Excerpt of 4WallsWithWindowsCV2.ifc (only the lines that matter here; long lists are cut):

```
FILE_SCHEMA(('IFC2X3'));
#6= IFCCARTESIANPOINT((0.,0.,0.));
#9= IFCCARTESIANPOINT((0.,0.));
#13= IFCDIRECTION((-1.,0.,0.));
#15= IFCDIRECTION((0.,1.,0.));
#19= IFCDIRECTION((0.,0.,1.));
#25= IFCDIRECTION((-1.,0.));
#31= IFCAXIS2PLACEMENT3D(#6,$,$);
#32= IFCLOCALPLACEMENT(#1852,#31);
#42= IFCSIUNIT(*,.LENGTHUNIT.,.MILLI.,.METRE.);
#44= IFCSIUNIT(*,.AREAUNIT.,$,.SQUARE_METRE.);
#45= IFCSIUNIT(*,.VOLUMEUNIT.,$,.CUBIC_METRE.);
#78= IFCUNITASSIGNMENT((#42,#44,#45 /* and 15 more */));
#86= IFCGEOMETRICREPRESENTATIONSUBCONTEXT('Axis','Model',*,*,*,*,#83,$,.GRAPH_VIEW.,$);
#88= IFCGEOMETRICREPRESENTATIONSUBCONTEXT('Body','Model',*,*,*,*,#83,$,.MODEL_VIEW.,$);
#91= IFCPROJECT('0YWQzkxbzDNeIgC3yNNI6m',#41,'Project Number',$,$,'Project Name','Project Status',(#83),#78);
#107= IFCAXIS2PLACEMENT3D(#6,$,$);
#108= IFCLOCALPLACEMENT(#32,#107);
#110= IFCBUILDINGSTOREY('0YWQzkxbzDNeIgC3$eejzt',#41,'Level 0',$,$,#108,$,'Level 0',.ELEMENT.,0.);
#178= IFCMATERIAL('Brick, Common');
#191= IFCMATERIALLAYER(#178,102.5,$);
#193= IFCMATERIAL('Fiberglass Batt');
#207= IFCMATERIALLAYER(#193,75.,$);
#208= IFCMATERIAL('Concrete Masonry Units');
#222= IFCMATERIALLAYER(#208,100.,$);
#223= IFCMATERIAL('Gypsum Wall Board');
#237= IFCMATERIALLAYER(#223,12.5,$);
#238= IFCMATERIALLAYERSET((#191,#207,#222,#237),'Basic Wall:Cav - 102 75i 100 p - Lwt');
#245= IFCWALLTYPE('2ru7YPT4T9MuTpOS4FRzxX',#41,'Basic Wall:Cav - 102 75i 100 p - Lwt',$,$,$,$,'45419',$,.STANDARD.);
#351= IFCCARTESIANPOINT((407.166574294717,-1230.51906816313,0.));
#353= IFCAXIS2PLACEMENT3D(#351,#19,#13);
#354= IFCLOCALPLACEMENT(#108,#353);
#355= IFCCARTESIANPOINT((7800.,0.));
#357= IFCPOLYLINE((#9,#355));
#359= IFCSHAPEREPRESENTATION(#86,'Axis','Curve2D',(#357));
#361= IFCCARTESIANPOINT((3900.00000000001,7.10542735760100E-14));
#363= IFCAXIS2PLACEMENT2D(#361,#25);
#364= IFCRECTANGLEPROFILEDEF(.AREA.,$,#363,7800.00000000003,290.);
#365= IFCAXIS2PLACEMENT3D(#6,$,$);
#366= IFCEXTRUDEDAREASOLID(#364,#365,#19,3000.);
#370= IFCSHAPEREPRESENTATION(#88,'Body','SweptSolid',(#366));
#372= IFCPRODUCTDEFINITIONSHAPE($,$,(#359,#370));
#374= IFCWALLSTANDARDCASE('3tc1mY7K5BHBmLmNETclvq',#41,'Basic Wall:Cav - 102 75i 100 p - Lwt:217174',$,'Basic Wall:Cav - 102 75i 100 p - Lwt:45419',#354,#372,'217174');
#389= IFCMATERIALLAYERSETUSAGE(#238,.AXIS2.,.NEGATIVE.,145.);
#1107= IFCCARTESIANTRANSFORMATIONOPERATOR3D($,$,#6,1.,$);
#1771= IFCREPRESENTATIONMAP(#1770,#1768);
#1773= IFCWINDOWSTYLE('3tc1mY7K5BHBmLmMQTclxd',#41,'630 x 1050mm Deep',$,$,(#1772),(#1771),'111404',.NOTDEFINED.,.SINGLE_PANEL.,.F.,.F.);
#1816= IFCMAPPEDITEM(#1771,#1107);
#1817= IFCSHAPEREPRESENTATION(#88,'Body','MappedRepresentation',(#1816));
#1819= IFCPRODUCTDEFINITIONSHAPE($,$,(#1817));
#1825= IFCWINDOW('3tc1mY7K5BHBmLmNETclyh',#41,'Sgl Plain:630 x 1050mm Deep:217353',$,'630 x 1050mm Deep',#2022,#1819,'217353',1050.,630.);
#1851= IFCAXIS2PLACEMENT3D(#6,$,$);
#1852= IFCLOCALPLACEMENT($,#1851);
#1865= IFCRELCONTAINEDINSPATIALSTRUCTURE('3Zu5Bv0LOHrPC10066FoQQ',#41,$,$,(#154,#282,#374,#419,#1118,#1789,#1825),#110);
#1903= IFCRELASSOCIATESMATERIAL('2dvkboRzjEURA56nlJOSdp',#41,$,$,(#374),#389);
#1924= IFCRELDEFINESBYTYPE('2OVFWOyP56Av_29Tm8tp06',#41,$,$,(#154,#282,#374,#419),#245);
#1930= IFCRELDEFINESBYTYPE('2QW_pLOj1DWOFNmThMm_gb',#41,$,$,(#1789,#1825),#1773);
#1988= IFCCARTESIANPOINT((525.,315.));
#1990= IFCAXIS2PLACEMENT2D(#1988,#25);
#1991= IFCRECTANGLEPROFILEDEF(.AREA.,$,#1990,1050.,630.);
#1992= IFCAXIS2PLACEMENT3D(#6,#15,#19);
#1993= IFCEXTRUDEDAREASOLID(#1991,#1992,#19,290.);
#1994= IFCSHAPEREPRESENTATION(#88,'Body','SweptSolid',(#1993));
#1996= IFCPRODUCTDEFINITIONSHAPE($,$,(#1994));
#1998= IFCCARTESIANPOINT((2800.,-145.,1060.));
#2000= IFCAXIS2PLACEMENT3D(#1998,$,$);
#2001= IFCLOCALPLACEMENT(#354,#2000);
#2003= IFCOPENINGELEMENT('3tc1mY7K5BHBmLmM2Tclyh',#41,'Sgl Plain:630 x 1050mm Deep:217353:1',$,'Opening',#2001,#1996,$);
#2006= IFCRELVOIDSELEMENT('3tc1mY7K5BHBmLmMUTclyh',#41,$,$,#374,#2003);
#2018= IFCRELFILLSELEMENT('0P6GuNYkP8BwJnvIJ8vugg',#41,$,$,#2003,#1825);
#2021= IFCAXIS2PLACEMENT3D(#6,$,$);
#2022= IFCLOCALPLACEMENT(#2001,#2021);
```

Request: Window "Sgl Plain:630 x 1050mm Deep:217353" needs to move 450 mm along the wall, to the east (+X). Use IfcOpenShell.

```python
import ifcopenshell
import ifcopenshell.api.geometry
import ifcopenshell.util.placement

model = ifcopenshell.open("4WallsWithWindowsCV2.ifc")

window = model.by_guid("3tc1mY7K5BHBmLmNETclyh")
opening = window.FillsVoids[0].RelatingOpeningElement
wall = opening.VoidsElements[0].RelatingBuildingElement

wall_matrix = ifcopenshell.util.placement.get_local_placement(wall.ObjectPlacement)
shift = wall_matrix[:3, 0] * -450.0
before = ifcopenshell.util.placement.get_local_placement(window.ObjectPlacement)[:3, 3].copy()

# The window is placed relative to its opening, so it follows when the opening moves.
matrix = ifcopenshell.util.placement.get_local_placement(opening.ObjectPlacement)
matrix[:3, 3] += shift
ifcopenshell.api.geometry.edit_object_placement(
    model, product=opening, matrix=matrix, is_si=False, should_transform_children=True
)

after = ifcopenshell.util.placement.get_local_placement(window.ObjectPlacement)[:3, 3]
print("window moved by", (after - before).round(3) + 0.0)

model.write("4WallsWithWindowsCV2_v2.ifc")
```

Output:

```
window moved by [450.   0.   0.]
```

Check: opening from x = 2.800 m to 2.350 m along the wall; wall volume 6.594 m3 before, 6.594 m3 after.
